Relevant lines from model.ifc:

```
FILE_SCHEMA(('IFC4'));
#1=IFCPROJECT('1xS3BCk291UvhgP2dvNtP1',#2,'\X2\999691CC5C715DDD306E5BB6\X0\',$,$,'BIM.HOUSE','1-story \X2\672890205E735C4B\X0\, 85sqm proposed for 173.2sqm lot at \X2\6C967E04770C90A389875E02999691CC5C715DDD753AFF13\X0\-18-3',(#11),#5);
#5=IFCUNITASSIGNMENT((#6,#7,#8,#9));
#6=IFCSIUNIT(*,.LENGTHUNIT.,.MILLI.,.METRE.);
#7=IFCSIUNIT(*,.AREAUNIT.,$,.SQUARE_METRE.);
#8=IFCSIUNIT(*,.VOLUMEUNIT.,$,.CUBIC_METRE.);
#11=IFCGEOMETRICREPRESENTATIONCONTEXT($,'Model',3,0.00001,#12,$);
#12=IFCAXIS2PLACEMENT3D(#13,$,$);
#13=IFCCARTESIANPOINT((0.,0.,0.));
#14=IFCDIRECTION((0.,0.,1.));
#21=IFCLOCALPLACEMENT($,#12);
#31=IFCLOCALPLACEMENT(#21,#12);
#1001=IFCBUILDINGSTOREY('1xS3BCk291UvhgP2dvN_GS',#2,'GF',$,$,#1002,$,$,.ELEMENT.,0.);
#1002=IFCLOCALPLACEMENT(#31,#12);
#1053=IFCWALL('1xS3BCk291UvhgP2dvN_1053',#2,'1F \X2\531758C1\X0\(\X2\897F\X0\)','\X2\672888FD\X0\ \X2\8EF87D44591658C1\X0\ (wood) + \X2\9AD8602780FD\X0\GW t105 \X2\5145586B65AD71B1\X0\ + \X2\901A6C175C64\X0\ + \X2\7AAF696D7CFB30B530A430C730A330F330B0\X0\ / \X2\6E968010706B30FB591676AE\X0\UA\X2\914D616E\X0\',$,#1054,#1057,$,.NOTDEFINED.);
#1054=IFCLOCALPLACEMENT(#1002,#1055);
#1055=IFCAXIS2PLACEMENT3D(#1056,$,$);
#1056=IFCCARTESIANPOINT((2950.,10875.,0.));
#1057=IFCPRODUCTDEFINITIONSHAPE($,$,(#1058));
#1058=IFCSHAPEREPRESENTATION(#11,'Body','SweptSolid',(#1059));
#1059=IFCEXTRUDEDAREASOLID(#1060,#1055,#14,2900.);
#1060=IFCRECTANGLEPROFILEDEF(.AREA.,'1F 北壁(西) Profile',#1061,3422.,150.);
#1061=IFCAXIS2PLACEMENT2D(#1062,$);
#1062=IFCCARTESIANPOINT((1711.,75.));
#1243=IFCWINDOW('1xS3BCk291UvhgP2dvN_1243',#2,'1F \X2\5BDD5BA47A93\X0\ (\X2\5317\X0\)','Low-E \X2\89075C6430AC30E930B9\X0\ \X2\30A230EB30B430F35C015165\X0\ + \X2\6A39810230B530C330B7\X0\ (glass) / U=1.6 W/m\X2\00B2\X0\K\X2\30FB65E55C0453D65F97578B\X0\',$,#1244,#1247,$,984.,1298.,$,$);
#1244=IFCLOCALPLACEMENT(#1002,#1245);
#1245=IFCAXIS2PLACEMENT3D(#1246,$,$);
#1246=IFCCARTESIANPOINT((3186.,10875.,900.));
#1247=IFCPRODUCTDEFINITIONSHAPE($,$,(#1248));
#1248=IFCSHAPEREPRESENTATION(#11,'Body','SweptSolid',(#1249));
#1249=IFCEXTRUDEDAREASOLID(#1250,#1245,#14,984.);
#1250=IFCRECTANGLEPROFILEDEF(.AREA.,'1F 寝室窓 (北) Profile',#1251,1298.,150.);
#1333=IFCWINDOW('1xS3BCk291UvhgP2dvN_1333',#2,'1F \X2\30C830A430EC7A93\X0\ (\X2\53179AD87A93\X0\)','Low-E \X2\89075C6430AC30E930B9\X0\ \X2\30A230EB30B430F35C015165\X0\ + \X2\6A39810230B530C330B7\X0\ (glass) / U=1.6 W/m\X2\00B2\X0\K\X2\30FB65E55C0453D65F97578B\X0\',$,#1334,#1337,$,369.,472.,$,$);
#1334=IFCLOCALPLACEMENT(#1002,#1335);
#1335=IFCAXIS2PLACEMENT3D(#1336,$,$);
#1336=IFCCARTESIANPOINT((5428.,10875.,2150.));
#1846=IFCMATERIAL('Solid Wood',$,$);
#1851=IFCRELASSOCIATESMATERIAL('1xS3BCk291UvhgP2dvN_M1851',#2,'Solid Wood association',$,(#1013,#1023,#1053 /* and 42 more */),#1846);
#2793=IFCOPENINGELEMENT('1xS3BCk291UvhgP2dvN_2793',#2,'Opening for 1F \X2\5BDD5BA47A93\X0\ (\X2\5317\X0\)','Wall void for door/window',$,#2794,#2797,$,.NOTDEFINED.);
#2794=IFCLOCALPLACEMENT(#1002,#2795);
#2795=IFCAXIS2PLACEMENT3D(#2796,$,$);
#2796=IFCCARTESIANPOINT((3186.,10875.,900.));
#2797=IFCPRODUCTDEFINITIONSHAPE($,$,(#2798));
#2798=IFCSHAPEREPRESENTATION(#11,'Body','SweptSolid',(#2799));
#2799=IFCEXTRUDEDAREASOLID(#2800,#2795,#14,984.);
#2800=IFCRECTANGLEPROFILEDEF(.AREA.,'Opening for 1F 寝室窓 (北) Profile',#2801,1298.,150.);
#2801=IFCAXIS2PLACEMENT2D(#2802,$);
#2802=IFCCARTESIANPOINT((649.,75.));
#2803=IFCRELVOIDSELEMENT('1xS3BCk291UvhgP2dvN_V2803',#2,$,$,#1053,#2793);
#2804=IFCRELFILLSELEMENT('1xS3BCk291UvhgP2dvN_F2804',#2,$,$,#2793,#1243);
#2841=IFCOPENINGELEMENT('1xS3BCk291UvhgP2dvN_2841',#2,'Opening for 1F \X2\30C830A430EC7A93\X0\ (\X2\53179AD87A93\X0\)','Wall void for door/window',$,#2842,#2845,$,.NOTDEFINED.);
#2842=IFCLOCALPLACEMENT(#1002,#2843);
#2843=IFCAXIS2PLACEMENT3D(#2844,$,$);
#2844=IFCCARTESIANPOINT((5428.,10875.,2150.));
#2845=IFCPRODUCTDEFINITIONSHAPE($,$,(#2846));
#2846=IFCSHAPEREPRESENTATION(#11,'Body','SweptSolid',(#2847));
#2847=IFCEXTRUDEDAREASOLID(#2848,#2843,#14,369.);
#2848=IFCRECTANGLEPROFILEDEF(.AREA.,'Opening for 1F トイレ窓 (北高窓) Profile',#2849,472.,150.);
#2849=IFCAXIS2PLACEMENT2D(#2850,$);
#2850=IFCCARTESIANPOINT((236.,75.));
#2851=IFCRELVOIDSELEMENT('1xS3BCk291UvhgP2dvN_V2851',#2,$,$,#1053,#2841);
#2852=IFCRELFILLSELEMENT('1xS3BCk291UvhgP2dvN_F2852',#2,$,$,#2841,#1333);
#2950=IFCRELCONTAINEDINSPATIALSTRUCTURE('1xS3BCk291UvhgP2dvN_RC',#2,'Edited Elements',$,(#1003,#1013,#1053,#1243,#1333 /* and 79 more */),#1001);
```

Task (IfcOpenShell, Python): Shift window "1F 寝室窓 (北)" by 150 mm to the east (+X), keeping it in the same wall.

```python
import ifcopenshell
import ifcopenshell.api.geometry
import ifcopenshell.util.placement

model = ifcopenshell.open("model.ifc")

window = model.by_guid("1xS3BCk291UvhgP2dvN_1243")
opening = window.FillsVoids[0].RelatingOpeningElement
wall = opening.VoidsElements[0].RelatingBuildingElement

wall_matrix = ifcopenshell.util.placement.get_local_placement(wall.ObjectPlacement)
shift = wall_matrix[:3, 0] * 150.0
before = ifcopenshell.util.placement.get_local_placement(window.ObjectPlacement)[:3, 3].copy()

# The window is not placed relative to its opening, so move both.
for product in (opening, window):
    matrix = ifcopenshell.util.placement.get_local_placement(product.ObjectPlacement)
    matrix[:3, 3] += shift
    ifcopenshell.api.geometry.edit_object_placement(model, product=product, matrix=matrix, is_si=False)

after = ifcopenshell.util.placement.get_local_placement(window.ObjectPlacement)[:3, 3]
print("window moved by", (after - before).round(3) + 0.0)

model.write("model_edited.ifc")
```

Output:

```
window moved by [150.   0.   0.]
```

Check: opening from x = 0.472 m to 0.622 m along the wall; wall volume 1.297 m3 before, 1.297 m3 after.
